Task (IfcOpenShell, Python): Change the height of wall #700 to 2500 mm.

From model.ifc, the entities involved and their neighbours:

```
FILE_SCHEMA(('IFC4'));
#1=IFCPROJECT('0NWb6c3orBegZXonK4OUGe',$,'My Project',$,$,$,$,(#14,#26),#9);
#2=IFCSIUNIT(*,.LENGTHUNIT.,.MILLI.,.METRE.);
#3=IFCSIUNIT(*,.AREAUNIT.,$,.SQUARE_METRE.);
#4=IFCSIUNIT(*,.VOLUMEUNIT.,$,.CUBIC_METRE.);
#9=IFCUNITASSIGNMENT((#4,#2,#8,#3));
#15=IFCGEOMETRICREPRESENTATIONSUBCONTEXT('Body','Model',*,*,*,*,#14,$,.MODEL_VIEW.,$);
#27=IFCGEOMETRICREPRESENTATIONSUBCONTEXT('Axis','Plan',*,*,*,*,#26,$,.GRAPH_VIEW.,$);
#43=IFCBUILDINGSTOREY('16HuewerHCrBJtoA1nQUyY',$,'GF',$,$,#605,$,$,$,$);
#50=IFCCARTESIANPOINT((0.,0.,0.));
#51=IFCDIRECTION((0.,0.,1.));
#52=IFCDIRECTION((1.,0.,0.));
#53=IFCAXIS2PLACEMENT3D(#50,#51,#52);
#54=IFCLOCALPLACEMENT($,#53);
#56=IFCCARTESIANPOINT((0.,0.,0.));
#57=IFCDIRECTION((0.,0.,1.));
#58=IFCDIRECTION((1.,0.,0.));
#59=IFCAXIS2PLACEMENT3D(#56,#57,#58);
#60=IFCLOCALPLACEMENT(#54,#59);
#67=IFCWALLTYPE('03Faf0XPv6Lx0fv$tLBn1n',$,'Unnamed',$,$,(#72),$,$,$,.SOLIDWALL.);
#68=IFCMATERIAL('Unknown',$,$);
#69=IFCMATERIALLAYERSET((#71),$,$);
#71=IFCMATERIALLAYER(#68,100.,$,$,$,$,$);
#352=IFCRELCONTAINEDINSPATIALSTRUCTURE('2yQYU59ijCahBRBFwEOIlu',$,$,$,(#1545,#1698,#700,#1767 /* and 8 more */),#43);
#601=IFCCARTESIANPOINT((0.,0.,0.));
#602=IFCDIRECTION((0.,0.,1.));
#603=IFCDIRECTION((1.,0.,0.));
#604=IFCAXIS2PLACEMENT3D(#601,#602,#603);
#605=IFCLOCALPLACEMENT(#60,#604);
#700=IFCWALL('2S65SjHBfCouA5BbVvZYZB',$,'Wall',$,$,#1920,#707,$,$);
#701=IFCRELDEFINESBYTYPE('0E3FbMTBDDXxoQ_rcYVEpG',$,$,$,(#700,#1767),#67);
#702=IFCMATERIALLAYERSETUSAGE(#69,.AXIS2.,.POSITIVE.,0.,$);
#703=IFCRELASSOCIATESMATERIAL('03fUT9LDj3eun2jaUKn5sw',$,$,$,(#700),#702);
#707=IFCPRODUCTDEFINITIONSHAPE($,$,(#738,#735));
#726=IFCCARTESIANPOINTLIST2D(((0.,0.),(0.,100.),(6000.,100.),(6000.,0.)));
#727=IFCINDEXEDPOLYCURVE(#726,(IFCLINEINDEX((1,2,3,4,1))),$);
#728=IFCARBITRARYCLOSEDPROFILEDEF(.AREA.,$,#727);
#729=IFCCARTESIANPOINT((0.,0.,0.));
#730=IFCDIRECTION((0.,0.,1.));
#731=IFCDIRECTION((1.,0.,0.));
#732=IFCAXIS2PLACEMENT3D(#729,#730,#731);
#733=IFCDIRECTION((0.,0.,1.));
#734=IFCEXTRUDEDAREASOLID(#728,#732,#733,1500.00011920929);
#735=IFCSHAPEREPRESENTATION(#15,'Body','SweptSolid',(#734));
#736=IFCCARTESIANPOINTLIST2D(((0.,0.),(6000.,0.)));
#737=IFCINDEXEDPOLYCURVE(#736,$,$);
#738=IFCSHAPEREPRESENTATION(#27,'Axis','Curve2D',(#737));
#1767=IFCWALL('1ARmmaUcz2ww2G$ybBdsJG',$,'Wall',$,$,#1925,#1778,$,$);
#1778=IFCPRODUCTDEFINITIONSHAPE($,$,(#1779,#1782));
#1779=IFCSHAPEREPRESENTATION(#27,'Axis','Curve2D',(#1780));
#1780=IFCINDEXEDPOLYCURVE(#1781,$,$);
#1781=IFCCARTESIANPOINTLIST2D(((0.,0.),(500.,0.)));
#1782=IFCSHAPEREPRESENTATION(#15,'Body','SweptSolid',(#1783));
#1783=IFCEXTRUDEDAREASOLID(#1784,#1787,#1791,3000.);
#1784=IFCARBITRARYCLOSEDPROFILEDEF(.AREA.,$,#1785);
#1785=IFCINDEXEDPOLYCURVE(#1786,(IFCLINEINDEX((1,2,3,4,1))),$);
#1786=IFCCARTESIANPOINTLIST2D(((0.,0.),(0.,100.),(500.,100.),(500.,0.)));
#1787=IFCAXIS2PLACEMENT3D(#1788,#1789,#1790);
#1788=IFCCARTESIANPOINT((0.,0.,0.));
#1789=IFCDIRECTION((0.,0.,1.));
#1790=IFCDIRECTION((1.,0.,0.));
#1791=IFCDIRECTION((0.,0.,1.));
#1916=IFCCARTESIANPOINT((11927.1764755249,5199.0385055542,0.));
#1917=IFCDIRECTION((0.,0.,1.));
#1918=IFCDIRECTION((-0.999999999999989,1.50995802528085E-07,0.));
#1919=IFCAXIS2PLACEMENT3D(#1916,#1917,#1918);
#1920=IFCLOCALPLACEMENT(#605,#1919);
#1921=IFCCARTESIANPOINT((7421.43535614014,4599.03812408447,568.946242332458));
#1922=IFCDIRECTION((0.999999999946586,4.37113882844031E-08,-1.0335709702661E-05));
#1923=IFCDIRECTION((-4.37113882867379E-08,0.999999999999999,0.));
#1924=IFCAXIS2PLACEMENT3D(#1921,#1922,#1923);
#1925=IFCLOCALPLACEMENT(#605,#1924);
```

```python
import ifcopenshell
import ifcopenshell.geom
import ifcopenshell.util.representation
import ifcopenshell.util.shape

model = ifcopenshell.open("model.ifc")
settings = ifcopenshell.geom.settings()


def volume(element):
    """Net volume in cubic metres, openings subtracted."""
    shape = ifcopenshell.geom.create_shape(settings, element)
    return ifcopenshell.util.shape.get_volume(shape.geometry)


wall = model.by_guid("2S65SjHBfCouA5BbVvZYZB")
before = volume(wall)

body = ifcopenshell.util.representation.get_representation(wall, "Model", "Body")
solid = body.Items[0]
old_height = solid.Depth
solid.Depth = 2500.0
after = volume(wall)

print(f"height {old_height:g} -> {solid.Depth:g}, volume {before:.3f} -> {after:.3f} m3")

model.write("model_v2.ifc")
```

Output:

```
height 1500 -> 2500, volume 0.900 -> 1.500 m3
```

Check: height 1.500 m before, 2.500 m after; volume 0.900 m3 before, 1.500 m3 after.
